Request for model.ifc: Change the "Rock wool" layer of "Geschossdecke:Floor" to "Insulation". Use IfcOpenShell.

First a look at what the model holds.

```python
import ifcopenshell
import ifcopenshell.util.element

model = ifcopenshell.open("model.ifc")
print(model.schema)
for layer_set in model.by_type("IfcMaterialLayerSet"):
    if layer_set.LayerSetName == "Geschossdecke:Floor":
        for layer in layer_set.MaterialLayers:
            print(layer.id(), layer.Material and layer.Material.Name, layer.LayerThickness, sep=" | ")
        print(len(ifcopenshell.util.element.get_elements_by_material(model, layer_set)), "elements and types use it")
print(sorted(m.Name for m in model.by_type("IfcMaterial") if m.Name)[:60])
```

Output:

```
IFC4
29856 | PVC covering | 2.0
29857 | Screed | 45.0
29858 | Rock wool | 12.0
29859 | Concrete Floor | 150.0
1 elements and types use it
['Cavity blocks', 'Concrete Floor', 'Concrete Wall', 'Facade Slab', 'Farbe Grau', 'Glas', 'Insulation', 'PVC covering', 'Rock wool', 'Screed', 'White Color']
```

```python
import ifcopenshell
import ifcopenshell.api.material

model = ifcopenshell.open("model.ifc")

layer_set = next(s for s in model.by_type("IfcMaterialLayerSet") if s.LayerSetName == "Geschossdecke:Floor")
layer = next(l for l in layer_set.MaterialLayers if l.Material and l.Material.Name == "Rock wool")
material = next(m for m in model.by_type("IfcMaterial") if m.Name == "Insulation")

# Point this one layer at the other material; renaming the old one would change it everywhere.
ifcopenshell.api.material.edit_layer(model, layer=layer, attributes={}, material=material)

print([l.Material.Name if l.Material else None for l in layer_set.MaterialLayers])

model.write("model_rev.ifc")
```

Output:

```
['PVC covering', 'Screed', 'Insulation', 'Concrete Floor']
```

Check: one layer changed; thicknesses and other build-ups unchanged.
